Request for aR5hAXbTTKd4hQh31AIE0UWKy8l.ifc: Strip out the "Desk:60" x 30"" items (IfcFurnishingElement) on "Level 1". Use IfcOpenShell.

First a look at what the model holds.

```python
import ifcopenshell
import ifcopenshell.util.element

model = ifcopenshell.open("aR5hAXbTTKd4hQh31AIE0UWKy8l.ifc")
print(model.schema)
storey = next(s for s in model.by_type("IfcBuildingStorey") if s.Name == "Level 1")
furniture = [e for e in ifcopenshell.util.element.get_decomposition(storey) if e.is_a("IfcFurnishingElement")]
seen = {}
for e in furniture:
    element_type = ifcopenshell.util.element.get_type(e)
    name = element_type.Name if element_type not in (None, e) else None
    seen[name] = seen.get(name, 0) + 1
for name, count in sorted(seen.items(), key=str):
    print(count, "x", name)
```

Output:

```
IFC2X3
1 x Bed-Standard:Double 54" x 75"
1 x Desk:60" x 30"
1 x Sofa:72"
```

```python
import ifcopenshell
import ifcopenshell.api.root
import ifcopenshell.util.element

model = ifcopenshell.open("aR5hAXbTTKd4hQh31AIE0UWKy8l.ifc")

storey = next(s for s in model.by_type("IfcBuildingStorey") if s.Name == "Level 1")
furniture = [e for e in ifcopenshell.util.element.get_decomposition(storey) if e.is_a("IfcFurnishingElement")]
targets = [e for e in furniture if (t := ifcopenshell.util.element.get_type(e)) not in (None, e) and t.Name == 'Desk:60" x 30"']

for e in targets:
    ifcopenshell.api.root.remove_product(model, product=e)
print(len(targets), "removed")

model.write("aR5hAXbTTKd4hQh31AIE0UWKy8l_updated.ifc")
```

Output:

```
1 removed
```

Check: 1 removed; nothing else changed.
